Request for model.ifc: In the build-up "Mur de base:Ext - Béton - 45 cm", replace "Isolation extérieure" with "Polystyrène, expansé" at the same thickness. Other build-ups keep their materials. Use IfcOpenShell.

First a look at what the model holds.

```python
import ifcopenshell
import ifcopenshell.util.element

model = ifcopenshell.open("model.ifc")
print(model.schema)
for layer_set in model.by_type("IfcMaterialLayerSet"):
    if layer_set.LayerSetName == "Mur de base:Ext - Béton - 45 cm":
        for layer in layer_set.MaterialLayers:
            print(layer.id(), layer.Material and layer.Material.Name, layer.LayerThickness, sep=" | ")
        print(len(ifcopenshell.util.element.get_elements_by_material(model, layer_set)), "elements and types use it")
print(sorted(m.Name for m in model.by_type("IfcMaterial") if m.Name)[:60])
```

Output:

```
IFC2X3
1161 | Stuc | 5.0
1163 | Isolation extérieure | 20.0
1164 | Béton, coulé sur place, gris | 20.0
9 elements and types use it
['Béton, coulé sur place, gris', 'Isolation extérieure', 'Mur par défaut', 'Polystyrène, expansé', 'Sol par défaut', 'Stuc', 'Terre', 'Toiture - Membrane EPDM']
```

```python
import ifcopenshell
import ifcopenshell.api.material

model = ifcopenshell.open("model.ifc")

layer_set = next(s for s in model.by_type("IfcMaterialLayerSet") if s.LayerSetName == "Mur de base:Ext - Béton - 45 cm")
layer = next(l for l in layer_set.MaterialLayers if l.Material and l.Material.Name == "Isolation extérieure")
material = next(m for m in model.by_type("IfcMaterial") if m.Name == "Polystyrène, expansé")

# Point this one layer at the other material; renaming the old one would change it everywhere.
ifcopenshell.api.material.edit_layer(model, layer=layer, attributes={}, material=material)

print([l.Material.Name if l.Material else None for l in layer_set.MaterialLayers])

model.write("model_rev.ifc")
```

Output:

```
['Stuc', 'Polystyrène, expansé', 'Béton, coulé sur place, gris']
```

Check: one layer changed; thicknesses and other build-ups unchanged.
